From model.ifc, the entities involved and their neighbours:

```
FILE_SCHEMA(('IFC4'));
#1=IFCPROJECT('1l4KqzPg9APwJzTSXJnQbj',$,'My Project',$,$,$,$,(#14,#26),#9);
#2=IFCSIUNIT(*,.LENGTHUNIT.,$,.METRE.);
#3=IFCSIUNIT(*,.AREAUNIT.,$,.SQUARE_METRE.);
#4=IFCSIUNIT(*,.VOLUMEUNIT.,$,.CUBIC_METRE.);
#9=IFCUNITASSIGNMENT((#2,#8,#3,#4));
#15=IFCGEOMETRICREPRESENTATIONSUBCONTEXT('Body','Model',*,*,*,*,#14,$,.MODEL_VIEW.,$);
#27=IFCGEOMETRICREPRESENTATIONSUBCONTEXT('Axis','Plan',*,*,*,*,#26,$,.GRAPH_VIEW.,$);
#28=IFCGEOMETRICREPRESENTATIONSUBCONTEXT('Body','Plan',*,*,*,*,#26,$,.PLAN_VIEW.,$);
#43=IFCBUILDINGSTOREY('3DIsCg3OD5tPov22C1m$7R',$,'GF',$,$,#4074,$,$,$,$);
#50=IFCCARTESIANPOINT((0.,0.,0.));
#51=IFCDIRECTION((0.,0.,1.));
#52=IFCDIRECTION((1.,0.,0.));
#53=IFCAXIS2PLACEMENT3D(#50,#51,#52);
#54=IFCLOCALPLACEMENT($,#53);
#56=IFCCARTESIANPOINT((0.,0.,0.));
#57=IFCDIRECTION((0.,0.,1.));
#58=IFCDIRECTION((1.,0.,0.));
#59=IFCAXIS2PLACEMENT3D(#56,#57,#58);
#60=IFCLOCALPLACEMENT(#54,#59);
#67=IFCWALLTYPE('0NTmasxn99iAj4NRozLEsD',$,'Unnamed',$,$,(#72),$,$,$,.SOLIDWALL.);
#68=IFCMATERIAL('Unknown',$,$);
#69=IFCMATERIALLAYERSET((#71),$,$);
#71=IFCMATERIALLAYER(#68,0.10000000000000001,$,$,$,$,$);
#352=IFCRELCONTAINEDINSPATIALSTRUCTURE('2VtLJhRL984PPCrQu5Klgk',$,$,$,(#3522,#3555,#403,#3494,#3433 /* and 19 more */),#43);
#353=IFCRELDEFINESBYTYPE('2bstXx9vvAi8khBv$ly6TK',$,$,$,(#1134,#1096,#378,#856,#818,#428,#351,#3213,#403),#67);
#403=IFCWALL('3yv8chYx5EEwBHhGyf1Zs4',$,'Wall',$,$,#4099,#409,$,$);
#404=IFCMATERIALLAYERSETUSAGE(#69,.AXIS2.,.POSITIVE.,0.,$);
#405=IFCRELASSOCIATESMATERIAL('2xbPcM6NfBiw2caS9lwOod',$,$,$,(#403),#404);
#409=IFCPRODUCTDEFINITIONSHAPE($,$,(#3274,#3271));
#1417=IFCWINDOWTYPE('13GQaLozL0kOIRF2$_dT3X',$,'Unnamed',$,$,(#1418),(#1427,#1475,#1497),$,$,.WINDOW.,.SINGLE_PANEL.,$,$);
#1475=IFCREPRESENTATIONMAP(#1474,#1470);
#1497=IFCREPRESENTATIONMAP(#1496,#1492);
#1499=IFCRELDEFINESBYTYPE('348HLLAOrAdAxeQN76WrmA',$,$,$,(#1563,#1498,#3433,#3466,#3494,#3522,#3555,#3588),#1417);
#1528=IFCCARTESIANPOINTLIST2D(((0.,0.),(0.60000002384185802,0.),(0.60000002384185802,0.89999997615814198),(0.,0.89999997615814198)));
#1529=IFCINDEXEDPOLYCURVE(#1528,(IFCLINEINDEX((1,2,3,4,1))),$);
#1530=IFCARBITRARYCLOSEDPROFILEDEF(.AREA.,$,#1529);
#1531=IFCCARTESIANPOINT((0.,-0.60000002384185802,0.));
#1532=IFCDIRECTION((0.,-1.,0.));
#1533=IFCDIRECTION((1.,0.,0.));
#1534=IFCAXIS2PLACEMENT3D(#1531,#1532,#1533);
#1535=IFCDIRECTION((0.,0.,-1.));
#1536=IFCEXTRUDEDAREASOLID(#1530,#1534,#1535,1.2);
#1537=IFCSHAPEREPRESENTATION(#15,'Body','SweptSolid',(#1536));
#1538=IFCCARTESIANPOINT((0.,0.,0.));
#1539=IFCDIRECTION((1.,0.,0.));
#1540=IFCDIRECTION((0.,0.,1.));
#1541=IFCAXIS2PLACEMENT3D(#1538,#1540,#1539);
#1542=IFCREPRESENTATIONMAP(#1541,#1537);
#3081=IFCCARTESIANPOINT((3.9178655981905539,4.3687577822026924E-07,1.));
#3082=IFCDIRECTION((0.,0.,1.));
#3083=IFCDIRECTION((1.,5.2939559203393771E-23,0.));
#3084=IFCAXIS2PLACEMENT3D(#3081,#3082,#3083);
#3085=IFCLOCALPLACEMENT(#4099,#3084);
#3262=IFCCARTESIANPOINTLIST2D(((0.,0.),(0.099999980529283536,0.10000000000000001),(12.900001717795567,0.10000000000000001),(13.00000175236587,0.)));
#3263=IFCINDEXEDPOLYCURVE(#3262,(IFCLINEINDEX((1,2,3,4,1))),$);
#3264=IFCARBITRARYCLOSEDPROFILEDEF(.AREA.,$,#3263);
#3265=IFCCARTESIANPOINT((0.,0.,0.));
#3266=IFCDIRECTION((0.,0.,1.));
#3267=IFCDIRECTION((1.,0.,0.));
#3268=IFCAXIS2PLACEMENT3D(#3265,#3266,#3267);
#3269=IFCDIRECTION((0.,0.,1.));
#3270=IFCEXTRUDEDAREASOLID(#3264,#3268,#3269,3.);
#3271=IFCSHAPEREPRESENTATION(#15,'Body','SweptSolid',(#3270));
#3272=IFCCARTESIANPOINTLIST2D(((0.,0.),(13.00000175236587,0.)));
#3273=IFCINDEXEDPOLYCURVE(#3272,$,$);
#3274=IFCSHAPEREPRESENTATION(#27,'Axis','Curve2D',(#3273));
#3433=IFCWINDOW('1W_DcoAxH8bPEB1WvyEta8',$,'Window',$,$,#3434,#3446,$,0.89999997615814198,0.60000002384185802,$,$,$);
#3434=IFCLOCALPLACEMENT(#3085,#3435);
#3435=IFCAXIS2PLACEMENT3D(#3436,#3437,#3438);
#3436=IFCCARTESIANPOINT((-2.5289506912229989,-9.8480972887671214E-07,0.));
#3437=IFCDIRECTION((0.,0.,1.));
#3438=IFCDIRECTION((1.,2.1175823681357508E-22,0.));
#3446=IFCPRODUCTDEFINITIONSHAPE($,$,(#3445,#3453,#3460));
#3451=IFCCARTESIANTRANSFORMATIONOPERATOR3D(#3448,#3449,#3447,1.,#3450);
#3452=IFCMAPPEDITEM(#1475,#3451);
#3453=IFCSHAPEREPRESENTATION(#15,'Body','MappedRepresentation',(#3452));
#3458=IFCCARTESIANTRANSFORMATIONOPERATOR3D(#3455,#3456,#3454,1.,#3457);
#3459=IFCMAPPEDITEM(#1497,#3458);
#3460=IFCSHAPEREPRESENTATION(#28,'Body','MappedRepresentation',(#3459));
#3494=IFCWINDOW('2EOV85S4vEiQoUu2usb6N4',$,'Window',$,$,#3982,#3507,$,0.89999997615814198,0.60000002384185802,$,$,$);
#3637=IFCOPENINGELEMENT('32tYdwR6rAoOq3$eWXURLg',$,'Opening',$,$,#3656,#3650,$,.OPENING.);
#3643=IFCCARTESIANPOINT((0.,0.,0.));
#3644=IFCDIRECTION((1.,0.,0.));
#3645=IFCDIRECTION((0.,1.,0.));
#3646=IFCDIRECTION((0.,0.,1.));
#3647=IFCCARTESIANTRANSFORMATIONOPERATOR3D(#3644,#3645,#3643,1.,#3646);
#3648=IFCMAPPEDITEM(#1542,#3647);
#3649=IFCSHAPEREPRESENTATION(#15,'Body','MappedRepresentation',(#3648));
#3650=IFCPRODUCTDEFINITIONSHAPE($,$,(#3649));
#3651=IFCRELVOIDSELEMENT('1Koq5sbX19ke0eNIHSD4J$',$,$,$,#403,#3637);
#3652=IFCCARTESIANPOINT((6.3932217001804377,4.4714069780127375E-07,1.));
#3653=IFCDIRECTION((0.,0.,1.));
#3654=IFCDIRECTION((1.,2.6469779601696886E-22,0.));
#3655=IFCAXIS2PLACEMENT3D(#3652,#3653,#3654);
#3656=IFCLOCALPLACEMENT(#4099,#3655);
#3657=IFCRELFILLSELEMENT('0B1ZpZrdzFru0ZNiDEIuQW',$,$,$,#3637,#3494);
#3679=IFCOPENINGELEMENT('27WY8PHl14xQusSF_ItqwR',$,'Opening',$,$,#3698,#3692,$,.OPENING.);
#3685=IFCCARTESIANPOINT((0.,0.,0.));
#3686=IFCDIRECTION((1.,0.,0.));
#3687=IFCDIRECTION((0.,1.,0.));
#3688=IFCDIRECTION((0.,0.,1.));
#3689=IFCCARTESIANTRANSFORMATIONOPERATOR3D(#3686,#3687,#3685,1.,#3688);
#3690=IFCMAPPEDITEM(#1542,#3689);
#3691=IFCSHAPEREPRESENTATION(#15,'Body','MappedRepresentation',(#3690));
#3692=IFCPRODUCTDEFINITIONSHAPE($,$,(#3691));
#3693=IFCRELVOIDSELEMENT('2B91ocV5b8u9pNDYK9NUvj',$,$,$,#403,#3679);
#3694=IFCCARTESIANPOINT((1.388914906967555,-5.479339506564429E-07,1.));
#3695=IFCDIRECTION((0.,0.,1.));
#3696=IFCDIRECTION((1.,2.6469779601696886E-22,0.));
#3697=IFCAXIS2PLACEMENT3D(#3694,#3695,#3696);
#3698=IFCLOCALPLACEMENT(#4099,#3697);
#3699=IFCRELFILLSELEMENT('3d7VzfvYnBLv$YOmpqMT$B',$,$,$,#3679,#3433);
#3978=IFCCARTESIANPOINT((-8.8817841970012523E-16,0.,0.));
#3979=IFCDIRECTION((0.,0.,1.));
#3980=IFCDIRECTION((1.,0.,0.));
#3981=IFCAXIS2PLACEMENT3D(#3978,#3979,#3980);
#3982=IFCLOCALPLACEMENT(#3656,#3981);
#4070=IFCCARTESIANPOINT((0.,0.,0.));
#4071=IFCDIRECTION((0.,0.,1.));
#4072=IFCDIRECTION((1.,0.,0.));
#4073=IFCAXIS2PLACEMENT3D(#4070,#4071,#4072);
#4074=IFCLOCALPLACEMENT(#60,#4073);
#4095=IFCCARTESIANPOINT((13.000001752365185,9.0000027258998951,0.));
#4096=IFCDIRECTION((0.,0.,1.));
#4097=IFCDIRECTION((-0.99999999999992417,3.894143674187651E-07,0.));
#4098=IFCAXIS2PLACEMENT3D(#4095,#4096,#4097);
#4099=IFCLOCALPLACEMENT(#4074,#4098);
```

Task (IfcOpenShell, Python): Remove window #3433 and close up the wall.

```python
import ifcopenshell
import ifcopenshell.api.feature
import ifcopenshell.api.root
import ifcopenshell.geom
import ifcopenshell.util.shape

model = ifcopenshell.open("model.ifc")
settings = ifcopenshell.geom.settings()


def volume(element):
    """Net volume in cubic metres, openings subtracted."""
    shape = ifcopenshell.geom.create_shape(settings, element)
    return ifcopenshell.util.shape.get_volume(shape.geometry)


window = model.by_id(3433)
opening = window.FillsVoids[0].RelatingOpeningElement
wall = opening.VoidsElements[0].RelatingBuildingElement
before = volume(wall)

ifcopenshell.api.root.remove_product(model, product=window)
ifcopenshell.api.feature.remove_feature(model, feature=opening)

after = volume(wall)

print(f"wall volume {before:.3f} -> {after:.3f} m3")

model.write("model-out.ifc")
```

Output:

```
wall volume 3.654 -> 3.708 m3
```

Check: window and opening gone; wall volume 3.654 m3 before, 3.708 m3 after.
